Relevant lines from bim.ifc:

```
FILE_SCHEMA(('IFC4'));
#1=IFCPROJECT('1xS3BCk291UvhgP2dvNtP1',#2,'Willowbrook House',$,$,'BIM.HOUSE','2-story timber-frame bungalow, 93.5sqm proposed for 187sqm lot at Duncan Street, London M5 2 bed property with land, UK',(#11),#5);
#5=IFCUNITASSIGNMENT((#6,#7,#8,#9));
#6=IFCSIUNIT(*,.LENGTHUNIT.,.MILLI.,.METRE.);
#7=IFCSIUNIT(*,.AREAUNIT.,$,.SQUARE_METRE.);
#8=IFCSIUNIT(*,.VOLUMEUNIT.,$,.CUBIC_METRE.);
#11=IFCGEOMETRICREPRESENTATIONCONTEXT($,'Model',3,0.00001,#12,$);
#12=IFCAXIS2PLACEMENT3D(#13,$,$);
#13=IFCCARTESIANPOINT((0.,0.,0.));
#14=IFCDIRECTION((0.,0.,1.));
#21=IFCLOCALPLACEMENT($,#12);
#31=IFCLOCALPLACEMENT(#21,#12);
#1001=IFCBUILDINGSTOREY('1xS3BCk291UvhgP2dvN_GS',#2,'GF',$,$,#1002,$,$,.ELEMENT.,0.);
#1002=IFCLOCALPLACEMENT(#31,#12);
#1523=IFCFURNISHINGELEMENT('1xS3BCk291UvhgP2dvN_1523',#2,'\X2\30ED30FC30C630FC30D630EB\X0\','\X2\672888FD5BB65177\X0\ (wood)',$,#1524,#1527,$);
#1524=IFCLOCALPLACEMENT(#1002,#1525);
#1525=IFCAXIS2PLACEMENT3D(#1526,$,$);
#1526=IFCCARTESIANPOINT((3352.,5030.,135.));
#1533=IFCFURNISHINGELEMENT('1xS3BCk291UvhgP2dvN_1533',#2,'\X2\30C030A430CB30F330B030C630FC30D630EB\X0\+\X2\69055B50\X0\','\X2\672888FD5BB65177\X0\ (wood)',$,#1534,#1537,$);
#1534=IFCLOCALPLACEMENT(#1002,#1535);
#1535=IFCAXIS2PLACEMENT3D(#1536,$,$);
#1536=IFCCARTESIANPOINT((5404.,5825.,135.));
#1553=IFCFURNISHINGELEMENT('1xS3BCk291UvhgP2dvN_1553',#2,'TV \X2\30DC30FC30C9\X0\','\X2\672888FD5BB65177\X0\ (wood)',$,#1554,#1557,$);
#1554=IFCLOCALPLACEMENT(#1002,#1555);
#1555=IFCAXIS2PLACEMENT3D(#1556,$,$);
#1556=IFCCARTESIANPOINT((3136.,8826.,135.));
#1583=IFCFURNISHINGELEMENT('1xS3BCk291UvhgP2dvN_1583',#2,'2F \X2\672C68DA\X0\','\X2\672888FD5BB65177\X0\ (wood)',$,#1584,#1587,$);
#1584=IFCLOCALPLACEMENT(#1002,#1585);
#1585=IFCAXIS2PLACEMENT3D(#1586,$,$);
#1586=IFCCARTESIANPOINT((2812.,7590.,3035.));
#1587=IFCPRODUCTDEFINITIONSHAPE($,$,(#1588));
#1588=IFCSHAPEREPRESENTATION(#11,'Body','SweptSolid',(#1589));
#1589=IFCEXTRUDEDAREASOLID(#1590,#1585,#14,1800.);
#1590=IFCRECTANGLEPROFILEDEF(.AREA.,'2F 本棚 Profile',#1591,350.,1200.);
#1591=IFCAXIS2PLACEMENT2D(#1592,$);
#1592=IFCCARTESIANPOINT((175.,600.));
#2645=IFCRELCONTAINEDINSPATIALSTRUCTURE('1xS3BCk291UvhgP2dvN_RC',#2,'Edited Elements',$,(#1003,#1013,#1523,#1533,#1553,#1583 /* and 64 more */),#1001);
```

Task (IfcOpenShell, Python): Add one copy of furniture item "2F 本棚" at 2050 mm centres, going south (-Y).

```python
import numpy as np
import ifcopenshell
import ifcopenshell.api.geometry
import ifcopenshell.api.root
import ifcopenshell.util.element
import ifcopenshell.util.placement
import ifcopenshell.util.unit

model = ifcopenshell.open("bim.ifc")
unit_scale = ifcopenshell.util.unit.calculate_unit_scale(model)


def reuse_history(source, copy):
    """copy_class also copies each property set's owner history, people and application; keep the originals."""
    for rel in copy.IsDefinedBy:
        if rel.is_a("IfcRelDefinesByProperties") and (history := rel.RelatingPropertyDefinition.OwnerHistory):
            rel.RelatingPropertyDefinition.OwnerHistory = source.OwnerHistory
            ifcopenshell.util.element.remove_deep2(model, history)


source = model.by_guid("1xS3BCk291UvhgP2dvN_1583")
base = ifcopenshell.util.placement.get_local_placement(source.ObjectPlacement)
step = np.array([0.0, -1.0, 0.0]) * 2.05 / unit_scale

for i in range(1, 2):
    copy = ifcopenshell.api.root.copy_class(model, product=source)
    copy.Representation = ifcopenshell.util.element.copy_deep(
        model, source.Representation, exclude=["IfcGeometricRepresentationContext", "IfcRepresentationMap"]
    )
    reuse_history(source, copy)
    matrix = base.copy()
    matrix[:3, 3] += i * step
    print("added at", matrix[:3, 3].round(3) + 0.0)
    ifcopenshell.api.geometry.edit_object_placement(model, product=copy, matrix=matrix, is_si=False)

model.write("bim_updated.ifc")
```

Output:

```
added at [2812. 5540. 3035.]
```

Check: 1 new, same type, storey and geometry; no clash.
